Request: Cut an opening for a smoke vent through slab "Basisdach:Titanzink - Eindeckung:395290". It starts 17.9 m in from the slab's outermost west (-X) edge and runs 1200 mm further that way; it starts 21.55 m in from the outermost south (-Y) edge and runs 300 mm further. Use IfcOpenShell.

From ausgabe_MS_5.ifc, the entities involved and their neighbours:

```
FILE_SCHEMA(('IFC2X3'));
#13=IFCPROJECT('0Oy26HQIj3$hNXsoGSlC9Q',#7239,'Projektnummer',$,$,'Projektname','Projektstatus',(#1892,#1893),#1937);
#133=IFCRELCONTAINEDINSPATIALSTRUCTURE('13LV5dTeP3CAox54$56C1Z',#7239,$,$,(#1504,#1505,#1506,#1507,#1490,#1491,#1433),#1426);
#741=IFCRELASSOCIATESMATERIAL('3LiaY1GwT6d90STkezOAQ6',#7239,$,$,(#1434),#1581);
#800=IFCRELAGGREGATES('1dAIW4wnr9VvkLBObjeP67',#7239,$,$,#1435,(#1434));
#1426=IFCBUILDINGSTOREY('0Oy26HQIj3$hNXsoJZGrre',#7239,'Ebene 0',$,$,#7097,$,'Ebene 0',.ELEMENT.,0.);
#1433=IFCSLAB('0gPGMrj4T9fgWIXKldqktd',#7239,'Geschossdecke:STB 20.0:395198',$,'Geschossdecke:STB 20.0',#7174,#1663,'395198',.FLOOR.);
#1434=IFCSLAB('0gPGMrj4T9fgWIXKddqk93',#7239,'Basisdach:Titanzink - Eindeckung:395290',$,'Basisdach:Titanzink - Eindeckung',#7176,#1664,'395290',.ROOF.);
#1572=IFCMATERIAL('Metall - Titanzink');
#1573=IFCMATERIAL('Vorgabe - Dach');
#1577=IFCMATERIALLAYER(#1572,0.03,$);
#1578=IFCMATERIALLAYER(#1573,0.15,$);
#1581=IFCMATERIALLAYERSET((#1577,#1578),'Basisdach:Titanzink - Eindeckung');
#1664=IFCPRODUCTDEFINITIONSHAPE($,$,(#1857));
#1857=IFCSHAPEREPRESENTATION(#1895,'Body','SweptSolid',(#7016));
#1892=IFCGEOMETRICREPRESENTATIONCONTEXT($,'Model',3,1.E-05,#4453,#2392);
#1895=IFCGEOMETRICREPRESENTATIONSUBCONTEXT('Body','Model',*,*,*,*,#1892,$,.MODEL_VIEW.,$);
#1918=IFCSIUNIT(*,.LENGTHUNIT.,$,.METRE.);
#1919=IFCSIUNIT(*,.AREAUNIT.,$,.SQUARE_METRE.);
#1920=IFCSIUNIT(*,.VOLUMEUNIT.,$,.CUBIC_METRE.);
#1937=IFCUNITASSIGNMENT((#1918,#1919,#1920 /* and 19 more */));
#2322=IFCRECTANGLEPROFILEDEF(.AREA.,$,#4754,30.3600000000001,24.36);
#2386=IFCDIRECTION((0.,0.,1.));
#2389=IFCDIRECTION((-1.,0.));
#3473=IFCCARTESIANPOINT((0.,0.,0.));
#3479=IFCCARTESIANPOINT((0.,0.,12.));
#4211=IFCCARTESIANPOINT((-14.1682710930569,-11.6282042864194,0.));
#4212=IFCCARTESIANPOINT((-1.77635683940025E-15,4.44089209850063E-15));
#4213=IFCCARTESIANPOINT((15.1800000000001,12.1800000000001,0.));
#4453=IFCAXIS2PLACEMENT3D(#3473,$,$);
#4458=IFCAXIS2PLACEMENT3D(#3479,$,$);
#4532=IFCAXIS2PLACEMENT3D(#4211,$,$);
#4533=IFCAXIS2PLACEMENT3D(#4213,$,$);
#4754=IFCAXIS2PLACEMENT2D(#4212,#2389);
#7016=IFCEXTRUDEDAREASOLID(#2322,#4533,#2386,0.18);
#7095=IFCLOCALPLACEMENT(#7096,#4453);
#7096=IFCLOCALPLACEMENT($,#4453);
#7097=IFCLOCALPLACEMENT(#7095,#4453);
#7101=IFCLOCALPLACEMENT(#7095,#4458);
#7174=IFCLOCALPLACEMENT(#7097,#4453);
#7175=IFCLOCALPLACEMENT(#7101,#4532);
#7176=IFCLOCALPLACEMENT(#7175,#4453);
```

```python
import numpy as np
import ifcopenshell
import ifcopenshell.api.feature
import ifcopenshell.api.geometry
import ifcopenshell.api.root
import ifcopenshell.geom
import ifcopenshell.util.placement
import ifcopenshell.util.representation
import ifcopenshell.util.shape
import ifcopenshell.util.unit

model = ifcopenshell.open("ausgabe_MS_5.ifc")
unit_scale = ifcopenshell.util.unit.calculate_unit_scale(model)
settings = ifcopenshell.geom.settings()


def volume(element):
    """Net volume in cubic metres, openings subtracted."""
    shape = ifcopenshell.geom.create_shape(settings, element)
    return ifcopenshell.util.shape.get_volume(shape.geometry)


slab = model.by_guid("0gPGMrj4T9fgWIXKddqk93")
before = volume(slab)

# Extent in the slab's own axes, in metres. The edges named are its -X and -Y sides.
slab_shape = ifcopenshell.geom.create_shape(settings, slab)
vertices = ifcopenshell.util.shape.get_vertices(slab_shape.geometry)
x_min, y_min, bottom = vertices.min(axis=0)
top = vertices[:, 2].max()

opening = ifcopenshell.api.root.create_entity(model, ifc_class="IfcOpeningElement", name="Smoke vent opening")
context = ifcopenshell.util.representation.get_context(model, "Model", "Body", "MODEL_VIEW")
width, depth = 1.2, 0.3
outline = [(0.0, 0.0), (width, 0.0), (width, depth), (0.0, depth), (0.0, 0.0)]
# Overshoot both faces by 50 mm so the cut is clean.
shape = ifcopenshell.api.geometry.add_slab_representation(
    model, context=context, depth=top - bottom + 0.1, polyline=outline
)
ifcopenshell.api.geometry.assign_representation(model, product=opening, representation=shape)

matrix = ifcopenshell.util.placement.get_local_placement(slab.ObjectPlacement)
matrix[:, 3] = matrix @ np.append(np.array([x_min + 17.9, y_min + 21.55, bottom - 0.05]) / unit_scale, 1.0)
ifcopenshell.api.geometry.edit_object_placement(model, product=opening, matrix=matrix, is_si=False)
ifcopenshell.api.feature.add_feature(model, feature=opening, element=slab)

after = volume(slab)

print(f"slab volume {before:.3f} -> {after:.3f} m3")

model.write("ausgabe_MS_5-out.ifc")
```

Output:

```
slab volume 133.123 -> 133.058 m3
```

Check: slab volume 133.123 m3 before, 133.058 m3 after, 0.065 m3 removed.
